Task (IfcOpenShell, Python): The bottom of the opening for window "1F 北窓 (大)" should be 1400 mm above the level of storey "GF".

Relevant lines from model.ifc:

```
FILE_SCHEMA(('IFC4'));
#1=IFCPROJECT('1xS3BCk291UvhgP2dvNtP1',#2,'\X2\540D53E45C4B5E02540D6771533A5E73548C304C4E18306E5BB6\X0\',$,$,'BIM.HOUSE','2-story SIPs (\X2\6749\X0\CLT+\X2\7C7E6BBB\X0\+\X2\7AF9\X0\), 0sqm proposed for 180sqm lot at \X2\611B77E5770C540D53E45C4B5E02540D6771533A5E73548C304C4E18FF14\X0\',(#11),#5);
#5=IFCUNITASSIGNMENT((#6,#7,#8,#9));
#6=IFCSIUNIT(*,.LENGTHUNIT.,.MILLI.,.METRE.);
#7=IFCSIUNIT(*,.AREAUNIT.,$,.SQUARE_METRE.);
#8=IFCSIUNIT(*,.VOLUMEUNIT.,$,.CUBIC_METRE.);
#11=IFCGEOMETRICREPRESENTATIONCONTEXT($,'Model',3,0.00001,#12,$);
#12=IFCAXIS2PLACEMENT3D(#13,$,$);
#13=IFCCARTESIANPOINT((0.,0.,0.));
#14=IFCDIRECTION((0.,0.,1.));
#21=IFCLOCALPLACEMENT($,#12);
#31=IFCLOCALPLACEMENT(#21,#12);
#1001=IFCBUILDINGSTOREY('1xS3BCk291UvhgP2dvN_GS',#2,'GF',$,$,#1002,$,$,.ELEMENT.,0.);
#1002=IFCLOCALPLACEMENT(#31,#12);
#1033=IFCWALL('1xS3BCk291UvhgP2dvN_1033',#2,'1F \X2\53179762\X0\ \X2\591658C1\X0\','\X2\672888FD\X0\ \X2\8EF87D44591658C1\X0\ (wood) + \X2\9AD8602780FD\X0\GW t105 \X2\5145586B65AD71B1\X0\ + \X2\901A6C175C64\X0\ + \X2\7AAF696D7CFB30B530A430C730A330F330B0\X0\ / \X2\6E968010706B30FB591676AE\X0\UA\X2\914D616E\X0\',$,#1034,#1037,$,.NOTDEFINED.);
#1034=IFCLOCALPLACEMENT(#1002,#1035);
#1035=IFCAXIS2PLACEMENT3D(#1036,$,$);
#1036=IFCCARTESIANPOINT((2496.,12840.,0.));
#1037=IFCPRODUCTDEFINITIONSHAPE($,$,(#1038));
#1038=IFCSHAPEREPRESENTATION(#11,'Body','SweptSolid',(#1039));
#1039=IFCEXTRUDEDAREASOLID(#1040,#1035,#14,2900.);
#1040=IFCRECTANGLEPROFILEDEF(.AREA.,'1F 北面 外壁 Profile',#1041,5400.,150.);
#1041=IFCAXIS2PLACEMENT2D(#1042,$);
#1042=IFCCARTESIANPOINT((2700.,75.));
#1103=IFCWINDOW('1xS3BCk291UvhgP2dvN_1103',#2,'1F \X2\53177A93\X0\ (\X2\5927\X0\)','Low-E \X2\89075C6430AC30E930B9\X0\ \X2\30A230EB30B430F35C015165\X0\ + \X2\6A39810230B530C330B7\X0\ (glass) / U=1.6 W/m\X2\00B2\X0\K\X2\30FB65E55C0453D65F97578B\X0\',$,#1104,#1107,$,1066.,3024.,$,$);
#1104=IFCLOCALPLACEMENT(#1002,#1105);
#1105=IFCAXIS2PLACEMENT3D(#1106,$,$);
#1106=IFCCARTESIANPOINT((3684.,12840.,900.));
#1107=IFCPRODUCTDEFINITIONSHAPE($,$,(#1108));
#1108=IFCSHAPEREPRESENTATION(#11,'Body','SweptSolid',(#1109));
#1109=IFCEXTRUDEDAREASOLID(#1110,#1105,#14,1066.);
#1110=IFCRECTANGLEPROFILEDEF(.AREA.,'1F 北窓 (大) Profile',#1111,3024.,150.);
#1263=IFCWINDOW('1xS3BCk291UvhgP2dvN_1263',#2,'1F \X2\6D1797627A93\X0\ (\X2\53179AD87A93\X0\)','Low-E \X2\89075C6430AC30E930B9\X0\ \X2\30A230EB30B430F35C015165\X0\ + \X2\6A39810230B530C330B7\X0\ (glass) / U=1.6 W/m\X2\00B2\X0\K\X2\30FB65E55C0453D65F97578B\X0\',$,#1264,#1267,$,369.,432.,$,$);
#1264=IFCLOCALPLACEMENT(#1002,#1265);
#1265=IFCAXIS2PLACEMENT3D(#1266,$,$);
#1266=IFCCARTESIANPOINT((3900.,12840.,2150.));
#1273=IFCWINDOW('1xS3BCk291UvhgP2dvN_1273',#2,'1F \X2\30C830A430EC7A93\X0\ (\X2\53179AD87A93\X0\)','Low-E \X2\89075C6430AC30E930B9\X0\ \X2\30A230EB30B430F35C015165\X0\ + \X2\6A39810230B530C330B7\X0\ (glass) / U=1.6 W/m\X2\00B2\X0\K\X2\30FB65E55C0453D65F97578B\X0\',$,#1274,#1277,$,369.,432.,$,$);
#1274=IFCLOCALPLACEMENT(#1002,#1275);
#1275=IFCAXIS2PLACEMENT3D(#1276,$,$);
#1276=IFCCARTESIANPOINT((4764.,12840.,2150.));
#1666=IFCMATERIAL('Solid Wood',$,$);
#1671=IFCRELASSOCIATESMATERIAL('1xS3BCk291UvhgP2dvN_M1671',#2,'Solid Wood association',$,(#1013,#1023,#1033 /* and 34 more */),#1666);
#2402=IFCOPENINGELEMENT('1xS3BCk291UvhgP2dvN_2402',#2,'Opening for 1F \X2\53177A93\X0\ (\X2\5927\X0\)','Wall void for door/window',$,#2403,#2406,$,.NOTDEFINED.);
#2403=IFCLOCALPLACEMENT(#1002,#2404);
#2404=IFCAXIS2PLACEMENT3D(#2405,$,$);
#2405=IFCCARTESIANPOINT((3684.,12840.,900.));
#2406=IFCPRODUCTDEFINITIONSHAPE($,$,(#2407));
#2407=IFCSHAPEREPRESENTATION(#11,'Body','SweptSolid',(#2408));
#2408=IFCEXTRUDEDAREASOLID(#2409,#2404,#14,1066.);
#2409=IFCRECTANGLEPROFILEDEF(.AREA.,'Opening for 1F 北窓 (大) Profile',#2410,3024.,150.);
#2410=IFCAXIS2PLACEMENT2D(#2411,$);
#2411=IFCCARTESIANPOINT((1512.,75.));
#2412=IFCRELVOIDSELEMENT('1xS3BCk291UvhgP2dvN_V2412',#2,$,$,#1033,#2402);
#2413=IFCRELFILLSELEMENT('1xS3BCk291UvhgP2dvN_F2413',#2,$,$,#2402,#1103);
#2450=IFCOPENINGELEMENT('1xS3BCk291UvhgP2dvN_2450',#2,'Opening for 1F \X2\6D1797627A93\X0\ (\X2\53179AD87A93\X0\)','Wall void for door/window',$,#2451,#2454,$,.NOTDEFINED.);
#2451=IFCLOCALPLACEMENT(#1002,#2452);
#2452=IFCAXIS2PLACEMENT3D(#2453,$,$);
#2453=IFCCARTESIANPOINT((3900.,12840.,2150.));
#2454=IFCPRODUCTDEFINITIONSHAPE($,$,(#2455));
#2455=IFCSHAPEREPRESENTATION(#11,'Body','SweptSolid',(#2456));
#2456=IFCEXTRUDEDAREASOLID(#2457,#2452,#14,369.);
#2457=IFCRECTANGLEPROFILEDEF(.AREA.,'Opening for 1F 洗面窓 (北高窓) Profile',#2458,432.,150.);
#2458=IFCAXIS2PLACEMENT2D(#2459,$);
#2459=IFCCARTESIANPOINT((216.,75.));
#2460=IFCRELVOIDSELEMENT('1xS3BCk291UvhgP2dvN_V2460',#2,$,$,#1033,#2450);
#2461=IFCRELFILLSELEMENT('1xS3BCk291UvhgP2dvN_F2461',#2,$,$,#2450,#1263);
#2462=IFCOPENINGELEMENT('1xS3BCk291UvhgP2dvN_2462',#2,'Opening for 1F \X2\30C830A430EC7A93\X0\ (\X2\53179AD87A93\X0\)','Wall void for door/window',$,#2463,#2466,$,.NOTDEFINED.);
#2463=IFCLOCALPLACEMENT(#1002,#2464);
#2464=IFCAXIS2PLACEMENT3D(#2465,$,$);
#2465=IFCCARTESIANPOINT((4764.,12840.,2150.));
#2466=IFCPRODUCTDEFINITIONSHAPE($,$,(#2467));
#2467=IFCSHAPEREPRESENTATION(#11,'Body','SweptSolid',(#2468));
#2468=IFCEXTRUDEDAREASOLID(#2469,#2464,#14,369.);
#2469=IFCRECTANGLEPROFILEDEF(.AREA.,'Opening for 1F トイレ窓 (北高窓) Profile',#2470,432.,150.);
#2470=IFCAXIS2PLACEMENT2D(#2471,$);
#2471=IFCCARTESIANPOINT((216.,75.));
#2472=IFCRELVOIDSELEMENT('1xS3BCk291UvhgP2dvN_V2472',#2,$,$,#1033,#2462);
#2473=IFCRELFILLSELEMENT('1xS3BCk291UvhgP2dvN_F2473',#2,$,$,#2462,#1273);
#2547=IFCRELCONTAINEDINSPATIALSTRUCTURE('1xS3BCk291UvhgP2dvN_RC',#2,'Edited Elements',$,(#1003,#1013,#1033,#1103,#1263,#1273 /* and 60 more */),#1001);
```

```python
import numpy as np
import ifcopenshell
import ifcopenshell.api.geometry
import ifcopenshell.geom
import ifcopenshell.util.element
import ifcopenshell.util.placement
import ifcopenshell.util.shape
import ifcopenshell.util.unit

model = ifcopenshell.open("model.ifc")
unit_scale = ifcopenshell.util.unit.calculate_unit_scale(model)

window = model.by_id(1103)
opening = window.FillsVoids[0].RelatingOpeningElement
storey = ifcopenshell.util.element.get_container(window, ifc_class="IfcBuildingStorey")
level = ifcopenshell.util.placement.get_local_placement(storey.ObjectPlacement)[2, 3]

# The opening's origin need not be at the sill, so measure its lowest point.
shape = ifcopenshell.geom.create_shape(ifcopenshell.geom.settings(), opening)
bottom = ifcopenshell.util.shape.get_shape_bottom_elevation(shape, shape.geometry) / unit_scale
dz = level + 1.4 / unit_scale - bottom

shift = np.array([0.0, 0.0, dz])
# The window is not placed relative to its opening, so move both.
for product in (opening, window):
    matrix = ifcopenshell.util.placement.get_local_placement(product.ObjectPlacement)
    matrix[:3, 3] += shift
    ifcopenshell.api.geometry.edit_object_placement(model, product=product, matrix=matrix, is_si=False)

print(f"moved by {dz * unit_scale:+.3f} m")

model.write("model_rev.ifc")
```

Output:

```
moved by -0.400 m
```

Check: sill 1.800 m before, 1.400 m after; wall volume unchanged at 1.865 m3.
